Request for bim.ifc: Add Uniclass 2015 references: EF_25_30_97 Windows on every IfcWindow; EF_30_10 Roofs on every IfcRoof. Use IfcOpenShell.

First a look at what the model holds.

```python
import ifcopenshell

model = ifcopenshell.open("bim.ifc")
print(model.schema)
print("classifications:", [c.Name for c in model.by_type("IfcClassification")])
for ifc_class in ("IfcDoor", "IfcRoof", "IfcStair", "IfcWall", "IfcWindow"):
    print(ifc_class, len(model.by_type(ifc_class)))
```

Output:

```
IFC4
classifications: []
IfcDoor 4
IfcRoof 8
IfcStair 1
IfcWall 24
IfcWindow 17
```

```python
import ifcopenshell
import ifcopenshell.api.classification

model = ifcopenshell.open("bim.ifc")

system = ifcopenshell.api.classification.add_classification(model, classification="Uniclass 2015")

codes = {
    "IfcWindow": ("EF_25_30_97", "Windows"),
    "IfcRoof": ("EF_30_10", "Roofs"),
}
for ifc_class, (code, name) in codes.items():
    products = model.by_type(ifc_class)
    ifcopenshell.api.classification.add_reference(
        model, products=products, classification=system, identification=code, name=name
    )
    print(code, len(products))

model.write("bim-out.ifc")
```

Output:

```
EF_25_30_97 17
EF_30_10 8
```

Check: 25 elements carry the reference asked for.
